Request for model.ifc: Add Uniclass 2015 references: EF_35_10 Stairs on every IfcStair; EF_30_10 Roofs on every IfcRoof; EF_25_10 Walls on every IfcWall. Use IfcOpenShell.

First a look at what the model holds.

```python
import ifcopenshell

model = ifcopenshell.open("model.ifc")
print(model.schema)
print("classifications:", [c.Name for c in model.by_type("IfcClassification")])
for ifc_class in ("IfcDoor", "IfcRoof", "IfcStair", "IfcWall", "IfcWindow"):
    print(ifc_class, len(model.by_type(ifc_class)))
```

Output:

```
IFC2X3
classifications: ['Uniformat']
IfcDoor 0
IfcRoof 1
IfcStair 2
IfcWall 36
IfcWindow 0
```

```python
import ifcopenshell
import ifcopenshell.api.classification

model = ifcopenshell.open("model.ifc")

# IFC2X3 requires Source and Edition and has no link from the project to the system.
system = model.create_entity("IfcClassification", Source="NBS", Edition="2015", Name="Uniclass 2015")

codes = {
    "IfcStair": ("EF_35_10", "Stairs"),
    "IfcRoof": ("EF_30_10", "Roofs"),
    "IfcWall": ("EF_25_10", "Walls"),
}
for ifc_class, (code, name) in codes.items():
    products = model.by_type(ifc_class)
    ifcopenshell.api.classification.add_reference(
        model, products=products, classification=system, identification=code, name=name
    )
    print(code, len(products))

model.write("model-out.ifc")
```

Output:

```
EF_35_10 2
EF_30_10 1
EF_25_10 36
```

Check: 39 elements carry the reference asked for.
